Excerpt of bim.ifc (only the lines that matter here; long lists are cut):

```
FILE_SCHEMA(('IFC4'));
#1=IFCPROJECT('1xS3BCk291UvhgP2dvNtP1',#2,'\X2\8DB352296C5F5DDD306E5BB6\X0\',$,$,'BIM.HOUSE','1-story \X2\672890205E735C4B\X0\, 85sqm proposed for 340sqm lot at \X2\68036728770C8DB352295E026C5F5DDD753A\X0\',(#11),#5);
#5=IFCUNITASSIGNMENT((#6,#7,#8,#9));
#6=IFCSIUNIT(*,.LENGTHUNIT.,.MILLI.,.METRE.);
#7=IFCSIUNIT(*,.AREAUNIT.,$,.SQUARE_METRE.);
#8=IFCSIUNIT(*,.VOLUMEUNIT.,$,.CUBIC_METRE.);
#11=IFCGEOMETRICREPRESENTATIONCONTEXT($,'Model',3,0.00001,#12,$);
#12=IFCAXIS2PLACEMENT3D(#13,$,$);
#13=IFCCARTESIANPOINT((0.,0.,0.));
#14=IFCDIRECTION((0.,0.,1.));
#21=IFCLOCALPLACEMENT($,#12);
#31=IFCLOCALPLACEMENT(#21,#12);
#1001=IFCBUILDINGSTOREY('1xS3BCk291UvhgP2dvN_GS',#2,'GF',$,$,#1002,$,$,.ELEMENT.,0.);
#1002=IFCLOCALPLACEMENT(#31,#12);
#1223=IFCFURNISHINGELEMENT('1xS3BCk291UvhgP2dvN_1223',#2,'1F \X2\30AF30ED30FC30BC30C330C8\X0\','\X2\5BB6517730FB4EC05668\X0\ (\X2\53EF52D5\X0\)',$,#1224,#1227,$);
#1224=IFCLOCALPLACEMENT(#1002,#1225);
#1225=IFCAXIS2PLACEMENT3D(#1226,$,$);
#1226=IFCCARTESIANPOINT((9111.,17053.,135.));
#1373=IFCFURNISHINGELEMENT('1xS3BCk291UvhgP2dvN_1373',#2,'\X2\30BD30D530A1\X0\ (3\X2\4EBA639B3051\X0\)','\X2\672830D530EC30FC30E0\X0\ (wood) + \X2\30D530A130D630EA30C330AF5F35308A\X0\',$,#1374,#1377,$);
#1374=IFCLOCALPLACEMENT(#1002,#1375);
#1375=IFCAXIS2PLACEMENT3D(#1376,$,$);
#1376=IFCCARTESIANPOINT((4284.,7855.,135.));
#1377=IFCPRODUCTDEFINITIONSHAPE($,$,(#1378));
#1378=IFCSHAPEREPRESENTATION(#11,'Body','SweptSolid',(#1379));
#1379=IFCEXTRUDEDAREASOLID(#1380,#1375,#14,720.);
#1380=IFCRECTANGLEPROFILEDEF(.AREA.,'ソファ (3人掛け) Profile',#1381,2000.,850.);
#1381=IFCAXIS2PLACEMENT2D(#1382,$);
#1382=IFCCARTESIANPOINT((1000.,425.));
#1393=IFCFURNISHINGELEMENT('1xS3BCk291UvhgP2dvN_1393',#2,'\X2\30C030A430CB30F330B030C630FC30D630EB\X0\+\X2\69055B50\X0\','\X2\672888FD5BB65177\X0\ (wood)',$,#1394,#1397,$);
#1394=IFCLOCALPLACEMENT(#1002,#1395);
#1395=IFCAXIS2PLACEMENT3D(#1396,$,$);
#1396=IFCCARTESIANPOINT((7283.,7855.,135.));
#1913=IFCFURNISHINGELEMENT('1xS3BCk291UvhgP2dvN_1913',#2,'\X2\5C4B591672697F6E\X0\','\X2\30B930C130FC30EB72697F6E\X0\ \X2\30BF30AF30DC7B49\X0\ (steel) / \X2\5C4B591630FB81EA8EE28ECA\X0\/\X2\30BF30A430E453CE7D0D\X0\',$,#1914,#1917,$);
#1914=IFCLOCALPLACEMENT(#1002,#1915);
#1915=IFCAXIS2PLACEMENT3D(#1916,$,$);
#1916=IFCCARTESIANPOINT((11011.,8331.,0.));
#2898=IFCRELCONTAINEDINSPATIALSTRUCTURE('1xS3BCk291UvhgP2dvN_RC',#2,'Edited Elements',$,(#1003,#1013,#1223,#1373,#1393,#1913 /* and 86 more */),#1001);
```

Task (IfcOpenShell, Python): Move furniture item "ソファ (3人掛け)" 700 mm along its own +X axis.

```python
import ifcopenshell
import ifcopenshell.api.geometry
import ifcopenshell.util.placement

model = ifcopenshell.open("bim.ifc")

item = model.by_guid("1xS3BCk291UvhgP2dvN_1373")
matrix = ifcopenshell.util.placement.get_local_placement(item.ObjectPlacement)
matrix[:3, 3] += matrix[:3, 0] * 700.0
ifcopenshell.api.geometry.edit_object_placement(model, product=item, matrix=matrix, is_si=False)

print(ifcopenshell.util.placement.get_local_placement(item.ObjectPlacement).round(3) + 0.0)

model.write("bim_v2.ifc")
```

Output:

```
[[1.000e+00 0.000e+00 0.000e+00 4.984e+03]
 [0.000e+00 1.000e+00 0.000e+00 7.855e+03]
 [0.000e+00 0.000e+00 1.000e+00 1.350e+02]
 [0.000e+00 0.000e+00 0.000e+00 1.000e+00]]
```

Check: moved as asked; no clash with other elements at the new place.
